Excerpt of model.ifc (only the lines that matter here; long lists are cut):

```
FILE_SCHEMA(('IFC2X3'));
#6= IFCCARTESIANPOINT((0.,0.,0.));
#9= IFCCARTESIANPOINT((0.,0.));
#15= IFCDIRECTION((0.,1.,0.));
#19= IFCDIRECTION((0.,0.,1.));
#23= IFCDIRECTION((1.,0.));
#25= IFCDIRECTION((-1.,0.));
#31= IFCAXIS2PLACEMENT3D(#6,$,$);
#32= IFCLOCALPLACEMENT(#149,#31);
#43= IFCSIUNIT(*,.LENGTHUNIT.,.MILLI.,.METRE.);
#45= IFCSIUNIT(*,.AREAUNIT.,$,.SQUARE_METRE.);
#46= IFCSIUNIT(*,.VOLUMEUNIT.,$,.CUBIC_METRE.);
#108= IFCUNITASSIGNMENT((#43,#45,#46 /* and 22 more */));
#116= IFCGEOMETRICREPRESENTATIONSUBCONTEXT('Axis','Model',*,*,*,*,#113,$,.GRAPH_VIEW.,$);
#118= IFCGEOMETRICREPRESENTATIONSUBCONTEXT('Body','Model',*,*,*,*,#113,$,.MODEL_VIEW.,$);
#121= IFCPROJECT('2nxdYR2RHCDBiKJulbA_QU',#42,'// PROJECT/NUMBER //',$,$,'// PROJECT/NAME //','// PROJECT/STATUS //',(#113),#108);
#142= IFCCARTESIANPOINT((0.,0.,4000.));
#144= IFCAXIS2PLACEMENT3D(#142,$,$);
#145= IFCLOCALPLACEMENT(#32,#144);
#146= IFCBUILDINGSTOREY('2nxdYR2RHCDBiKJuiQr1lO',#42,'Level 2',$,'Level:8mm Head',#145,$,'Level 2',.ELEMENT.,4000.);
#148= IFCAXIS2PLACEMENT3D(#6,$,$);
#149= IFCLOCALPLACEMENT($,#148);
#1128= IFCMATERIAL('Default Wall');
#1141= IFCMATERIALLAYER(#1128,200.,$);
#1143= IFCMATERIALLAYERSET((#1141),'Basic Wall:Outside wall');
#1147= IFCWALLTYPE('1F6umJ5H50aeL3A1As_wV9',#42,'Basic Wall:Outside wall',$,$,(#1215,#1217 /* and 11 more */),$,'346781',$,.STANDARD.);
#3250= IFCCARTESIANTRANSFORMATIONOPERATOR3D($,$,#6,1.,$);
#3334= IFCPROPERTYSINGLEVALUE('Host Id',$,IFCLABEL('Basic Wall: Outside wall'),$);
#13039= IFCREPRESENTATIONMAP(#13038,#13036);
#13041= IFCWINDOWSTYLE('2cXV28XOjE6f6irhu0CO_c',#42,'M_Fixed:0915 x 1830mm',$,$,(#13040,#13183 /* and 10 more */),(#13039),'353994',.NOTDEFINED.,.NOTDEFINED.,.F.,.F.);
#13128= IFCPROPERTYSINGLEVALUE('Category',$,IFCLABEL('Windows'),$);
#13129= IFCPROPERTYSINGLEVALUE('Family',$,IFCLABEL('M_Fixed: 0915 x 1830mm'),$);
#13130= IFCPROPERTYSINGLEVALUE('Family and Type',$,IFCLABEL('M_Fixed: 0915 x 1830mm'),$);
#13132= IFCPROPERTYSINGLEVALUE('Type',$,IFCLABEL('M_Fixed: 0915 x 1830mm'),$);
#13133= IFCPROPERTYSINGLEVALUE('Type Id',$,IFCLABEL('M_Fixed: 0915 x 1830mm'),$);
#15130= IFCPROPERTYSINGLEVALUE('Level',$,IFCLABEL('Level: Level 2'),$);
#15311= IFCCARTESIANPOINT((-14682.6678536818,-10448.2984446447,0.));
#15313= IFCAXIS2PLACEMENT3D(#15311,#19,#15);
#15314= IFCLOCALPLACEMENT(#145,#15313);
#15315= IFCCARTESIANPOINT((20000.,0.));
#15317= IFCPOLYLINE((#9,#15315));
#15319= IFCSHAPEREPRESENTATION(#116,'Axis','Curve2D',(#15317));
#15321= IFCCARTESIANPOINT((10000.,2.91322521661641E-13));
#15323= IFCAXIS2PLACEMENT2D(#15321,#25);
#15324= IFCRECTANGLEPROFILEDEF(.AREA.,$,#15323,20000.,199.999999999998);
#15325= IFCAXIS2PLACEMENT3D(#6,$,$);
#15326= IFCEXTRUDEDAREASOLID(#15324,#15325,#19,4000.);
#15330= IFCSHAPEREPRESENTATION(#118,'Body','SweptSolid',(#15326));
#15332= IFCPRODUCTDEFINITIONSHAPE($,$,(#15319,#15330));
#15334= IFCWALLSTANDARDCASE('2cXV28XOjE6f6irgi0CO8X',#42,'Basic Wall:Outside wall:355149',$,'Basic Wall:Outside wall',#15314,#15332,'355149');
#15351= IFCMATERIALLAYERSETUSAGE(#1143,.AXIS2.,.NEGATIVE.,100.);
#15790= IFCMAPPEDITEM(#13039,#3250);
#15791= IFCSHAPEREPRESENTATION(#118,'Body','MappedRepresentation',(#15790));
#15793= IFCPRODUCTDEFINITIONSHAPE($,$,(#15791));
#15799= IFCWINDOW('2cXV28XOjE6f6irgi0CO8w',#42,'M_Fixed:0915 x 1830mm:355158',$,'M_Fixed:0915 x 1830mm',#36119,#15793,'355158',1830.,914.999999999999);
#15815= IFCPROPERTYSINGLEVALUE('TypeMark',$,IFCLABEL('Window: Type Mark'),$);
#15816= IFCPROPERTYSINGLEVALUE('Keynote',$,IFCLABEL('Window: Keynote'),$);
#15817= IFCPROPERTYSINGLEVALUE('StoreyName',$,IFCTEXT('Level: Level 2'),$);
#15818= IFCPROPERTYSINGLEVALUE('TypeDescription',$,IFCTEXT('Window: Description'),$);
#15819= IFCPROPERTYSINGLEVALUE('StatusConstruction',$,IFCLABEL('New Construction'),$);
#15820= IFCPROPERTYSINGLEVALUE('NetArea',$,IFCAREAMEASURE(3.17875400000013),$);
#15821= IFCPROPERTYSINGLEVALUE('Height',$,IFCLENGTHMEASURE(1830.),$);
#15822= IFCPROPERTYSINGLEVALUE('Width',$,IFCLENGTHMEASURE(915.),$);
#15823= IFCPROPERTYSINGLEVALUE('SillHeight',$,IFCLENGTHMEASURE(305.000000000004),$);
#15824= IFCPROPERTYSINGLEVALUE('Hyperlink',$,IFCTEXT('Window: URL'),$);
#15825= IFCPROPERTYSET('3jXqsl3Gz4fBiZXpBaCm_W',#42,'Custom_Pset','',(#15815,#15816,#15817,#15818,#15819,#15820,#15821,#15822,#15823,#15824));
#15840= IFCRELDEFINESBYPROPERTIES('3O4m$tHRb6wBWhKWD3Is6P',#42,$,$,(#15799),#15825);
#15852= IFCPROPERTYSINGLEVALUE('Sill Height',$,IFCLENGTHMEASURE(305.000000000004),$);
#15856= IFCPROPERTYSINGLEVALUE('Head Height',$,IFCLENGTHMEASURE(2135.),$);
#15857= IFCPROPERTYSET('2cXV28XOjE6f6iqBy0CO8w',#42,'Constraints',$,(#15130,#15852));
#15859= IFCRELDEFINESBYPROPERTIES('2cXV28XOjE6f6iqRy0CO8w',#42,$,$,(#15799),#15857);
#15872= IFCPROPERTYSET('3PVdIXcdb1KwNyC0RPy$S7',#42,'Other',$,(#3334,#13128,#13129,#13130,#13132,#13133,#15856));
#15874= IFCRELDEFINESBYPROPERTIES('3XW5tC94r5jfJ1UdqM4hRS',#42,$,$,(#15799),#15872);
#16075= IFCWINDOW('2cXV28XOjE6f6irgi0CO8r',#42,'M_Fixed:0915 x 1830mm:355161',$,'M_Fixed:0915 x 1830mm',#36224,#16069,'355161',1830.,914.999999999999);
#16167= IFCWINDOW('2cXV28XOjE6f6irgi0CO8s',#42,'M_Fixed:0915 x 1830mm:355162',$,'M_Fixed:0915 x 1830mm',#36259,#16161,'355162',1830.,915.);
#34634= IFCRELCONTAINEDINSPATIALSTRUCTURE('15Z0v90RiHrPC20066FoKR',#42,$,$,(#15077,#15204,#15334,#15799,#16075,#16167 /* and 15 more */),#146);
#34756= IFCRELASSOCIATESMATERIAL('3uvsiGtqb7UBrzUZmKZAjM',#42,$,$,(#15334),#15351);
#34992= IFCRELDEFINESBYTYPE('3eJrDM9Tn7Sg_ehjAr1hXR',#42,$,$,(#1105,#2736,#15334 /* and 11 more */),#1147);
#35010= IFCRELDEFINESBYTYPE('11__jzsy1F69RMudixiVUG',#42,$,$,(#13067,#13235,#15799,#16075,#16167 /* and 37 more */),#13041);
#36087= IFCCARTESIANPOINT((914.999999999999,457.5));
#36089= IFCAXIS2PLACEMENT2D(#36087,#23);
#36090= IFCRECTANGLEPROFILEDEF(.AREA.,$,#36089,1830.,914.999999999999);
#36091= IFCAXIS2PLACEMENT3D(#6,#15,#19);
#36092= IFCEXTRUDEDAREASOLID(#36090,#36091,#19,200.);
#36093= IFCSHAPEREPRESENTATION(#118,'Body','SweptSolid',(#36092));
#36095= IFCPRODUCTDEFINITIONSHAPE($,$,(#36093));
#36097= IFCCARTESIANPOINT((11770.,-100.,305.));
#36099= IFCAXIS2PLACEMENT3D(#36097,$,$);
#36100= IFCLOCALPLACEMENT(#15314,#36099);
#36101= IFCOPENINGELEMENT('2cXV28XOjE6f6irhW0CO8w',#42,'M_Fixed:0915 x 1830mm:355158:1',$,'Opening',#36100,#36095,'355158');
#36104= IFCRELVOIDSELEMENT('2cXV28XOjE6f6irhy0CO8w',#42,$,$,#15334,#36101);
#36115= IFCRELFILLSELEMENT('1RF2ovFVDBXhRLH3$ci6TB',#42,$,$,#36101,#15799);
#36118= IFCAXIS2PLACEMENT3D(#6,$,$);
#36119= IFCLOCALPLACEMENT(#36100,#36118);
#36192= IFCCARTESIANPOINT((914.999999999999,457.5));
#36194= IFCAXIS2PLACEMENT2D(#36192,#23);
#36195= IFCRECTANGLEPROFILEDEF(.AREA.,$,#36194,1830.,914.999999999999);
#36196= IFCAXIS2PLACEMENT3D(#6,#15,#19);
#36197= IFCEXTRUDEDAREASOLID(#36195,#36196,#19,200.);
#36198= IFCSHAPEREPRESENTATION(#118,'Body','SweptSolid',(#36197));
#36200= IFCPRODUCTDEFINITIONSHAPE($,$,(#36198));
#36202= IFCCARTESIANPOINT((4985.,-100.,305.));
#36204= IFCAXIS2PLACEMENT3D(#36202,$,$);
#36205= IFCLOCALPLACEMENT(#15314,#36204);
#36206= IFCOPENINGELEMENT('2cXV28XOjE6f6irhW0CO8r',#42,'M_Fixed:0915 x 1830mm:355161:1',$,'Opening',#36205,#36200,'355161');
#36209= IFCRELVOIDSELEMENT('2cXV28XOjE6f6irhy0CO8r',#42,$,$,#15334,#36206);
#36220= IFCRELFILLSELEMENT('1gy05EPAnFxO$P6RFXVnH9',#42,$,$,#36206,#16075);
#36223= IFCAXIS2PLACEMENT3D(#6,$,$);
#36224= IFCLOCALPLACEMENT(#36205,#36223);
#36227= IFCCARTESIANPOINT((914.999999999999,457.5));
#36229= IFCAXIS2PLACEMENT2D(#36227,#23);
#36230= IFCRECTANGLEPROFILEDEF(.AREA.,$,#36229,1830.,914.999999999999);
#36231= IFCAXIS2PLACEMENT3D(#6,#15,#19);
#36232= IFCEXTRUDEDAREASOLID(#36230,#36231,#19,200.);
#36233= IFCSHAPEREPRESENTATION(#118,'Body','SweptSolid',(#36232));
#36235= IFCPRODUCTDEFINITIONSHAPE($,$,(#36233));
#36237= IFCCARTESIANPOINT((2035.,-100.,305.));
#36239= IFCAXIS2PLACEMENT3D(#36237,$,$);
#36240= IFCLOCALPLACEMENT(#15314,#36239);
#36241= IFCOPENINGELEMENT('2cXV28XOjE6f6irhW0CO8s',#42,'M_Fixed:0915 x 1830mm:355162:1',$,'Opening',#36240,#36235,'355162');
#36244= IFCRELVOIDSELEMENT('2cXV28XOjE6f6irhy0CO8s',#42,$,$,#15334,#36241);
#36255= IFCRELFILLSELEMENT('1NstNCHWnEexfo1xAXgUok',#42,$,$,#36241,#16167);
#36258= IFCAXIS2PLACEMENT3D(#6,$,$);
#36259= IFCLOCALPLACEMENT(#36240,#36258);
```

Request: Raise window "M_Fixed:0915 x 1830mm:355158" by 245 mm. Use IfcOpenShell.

```python
import numpy as np
import ifcopenshell
import ifcopenshell.api.geometry
import ifcopenshell.api.pset
import ifcopenshell.util.element
import ifcopenshell.util.placement
import ifcopenshell.util.unit

model = ifcopenshell.open("model.ifc")
unit_scale = ifcopenshell.util.unit.calculate_unit_scale(model)

window = model.by_guid("2cXV28XOjE6f6irgi0CO8w")
opening = window.FillsVoids[0].RelatingOpeningElement
dz = 0.245 / unit_scale

shift = np.array([0.0, 0.0, dz])
# The window is placed relative to its opening, so it follows when the opening moves.
matrix = ifcopenshell.util.placement.get_local_placement(opening.ObjectPlacement)
matrix[:3, 3] += shift
ifcopenshell.api.geometry.edit_object_placement(
    model, product=opening, matrix=matrix, is_si=False, should_transform_children=True
)

# Keep the stored heights in step.
pset = model.by_id(ifcopenshell.util.element.get_pset(window, "Custom_Pset", should_inherit=False)["id"])
ifcopenshell.api.pset.edit_pset(model, pset=pset, properties={
    "SillHeight": model.create_entity("IfcLengthMeasure", ifcopenshell.util.element.get_pset(window, "Constraints", "Sill Height") + dz),
})
pset = model.by_id(ifcopenshell.util.element.get_pset(window, "Constraints", should_inherit=False)["id"])
ifcopenshell.api.pset.edit_pset(model, pset=pset, properties={
    "Sill Height": model.create_entity("IfcLengthMeasure", ifcopenshell.util.element.get_pset(window, "Constraints", "Sill Height") + dz),
})
pset = model.by_id(ifcopenshell.util.element.get_pset(window, "Other", should_inherit=False)["id"])
ifcopenshell.api.pset.edit_pset(model, pset=pset, properties={
    "Head Height": model.create_entity("IfcLengthMeasure", ifcopenshell.util.element.get_pset(window, "Other", "Head Height") + dz),
})

print(f"moved by {dz * unit_scale:+.3f} m")

model.write("model-out.ifc")
```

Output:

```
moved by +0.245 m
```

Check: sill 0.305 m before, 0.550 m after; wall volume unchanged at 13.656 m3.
